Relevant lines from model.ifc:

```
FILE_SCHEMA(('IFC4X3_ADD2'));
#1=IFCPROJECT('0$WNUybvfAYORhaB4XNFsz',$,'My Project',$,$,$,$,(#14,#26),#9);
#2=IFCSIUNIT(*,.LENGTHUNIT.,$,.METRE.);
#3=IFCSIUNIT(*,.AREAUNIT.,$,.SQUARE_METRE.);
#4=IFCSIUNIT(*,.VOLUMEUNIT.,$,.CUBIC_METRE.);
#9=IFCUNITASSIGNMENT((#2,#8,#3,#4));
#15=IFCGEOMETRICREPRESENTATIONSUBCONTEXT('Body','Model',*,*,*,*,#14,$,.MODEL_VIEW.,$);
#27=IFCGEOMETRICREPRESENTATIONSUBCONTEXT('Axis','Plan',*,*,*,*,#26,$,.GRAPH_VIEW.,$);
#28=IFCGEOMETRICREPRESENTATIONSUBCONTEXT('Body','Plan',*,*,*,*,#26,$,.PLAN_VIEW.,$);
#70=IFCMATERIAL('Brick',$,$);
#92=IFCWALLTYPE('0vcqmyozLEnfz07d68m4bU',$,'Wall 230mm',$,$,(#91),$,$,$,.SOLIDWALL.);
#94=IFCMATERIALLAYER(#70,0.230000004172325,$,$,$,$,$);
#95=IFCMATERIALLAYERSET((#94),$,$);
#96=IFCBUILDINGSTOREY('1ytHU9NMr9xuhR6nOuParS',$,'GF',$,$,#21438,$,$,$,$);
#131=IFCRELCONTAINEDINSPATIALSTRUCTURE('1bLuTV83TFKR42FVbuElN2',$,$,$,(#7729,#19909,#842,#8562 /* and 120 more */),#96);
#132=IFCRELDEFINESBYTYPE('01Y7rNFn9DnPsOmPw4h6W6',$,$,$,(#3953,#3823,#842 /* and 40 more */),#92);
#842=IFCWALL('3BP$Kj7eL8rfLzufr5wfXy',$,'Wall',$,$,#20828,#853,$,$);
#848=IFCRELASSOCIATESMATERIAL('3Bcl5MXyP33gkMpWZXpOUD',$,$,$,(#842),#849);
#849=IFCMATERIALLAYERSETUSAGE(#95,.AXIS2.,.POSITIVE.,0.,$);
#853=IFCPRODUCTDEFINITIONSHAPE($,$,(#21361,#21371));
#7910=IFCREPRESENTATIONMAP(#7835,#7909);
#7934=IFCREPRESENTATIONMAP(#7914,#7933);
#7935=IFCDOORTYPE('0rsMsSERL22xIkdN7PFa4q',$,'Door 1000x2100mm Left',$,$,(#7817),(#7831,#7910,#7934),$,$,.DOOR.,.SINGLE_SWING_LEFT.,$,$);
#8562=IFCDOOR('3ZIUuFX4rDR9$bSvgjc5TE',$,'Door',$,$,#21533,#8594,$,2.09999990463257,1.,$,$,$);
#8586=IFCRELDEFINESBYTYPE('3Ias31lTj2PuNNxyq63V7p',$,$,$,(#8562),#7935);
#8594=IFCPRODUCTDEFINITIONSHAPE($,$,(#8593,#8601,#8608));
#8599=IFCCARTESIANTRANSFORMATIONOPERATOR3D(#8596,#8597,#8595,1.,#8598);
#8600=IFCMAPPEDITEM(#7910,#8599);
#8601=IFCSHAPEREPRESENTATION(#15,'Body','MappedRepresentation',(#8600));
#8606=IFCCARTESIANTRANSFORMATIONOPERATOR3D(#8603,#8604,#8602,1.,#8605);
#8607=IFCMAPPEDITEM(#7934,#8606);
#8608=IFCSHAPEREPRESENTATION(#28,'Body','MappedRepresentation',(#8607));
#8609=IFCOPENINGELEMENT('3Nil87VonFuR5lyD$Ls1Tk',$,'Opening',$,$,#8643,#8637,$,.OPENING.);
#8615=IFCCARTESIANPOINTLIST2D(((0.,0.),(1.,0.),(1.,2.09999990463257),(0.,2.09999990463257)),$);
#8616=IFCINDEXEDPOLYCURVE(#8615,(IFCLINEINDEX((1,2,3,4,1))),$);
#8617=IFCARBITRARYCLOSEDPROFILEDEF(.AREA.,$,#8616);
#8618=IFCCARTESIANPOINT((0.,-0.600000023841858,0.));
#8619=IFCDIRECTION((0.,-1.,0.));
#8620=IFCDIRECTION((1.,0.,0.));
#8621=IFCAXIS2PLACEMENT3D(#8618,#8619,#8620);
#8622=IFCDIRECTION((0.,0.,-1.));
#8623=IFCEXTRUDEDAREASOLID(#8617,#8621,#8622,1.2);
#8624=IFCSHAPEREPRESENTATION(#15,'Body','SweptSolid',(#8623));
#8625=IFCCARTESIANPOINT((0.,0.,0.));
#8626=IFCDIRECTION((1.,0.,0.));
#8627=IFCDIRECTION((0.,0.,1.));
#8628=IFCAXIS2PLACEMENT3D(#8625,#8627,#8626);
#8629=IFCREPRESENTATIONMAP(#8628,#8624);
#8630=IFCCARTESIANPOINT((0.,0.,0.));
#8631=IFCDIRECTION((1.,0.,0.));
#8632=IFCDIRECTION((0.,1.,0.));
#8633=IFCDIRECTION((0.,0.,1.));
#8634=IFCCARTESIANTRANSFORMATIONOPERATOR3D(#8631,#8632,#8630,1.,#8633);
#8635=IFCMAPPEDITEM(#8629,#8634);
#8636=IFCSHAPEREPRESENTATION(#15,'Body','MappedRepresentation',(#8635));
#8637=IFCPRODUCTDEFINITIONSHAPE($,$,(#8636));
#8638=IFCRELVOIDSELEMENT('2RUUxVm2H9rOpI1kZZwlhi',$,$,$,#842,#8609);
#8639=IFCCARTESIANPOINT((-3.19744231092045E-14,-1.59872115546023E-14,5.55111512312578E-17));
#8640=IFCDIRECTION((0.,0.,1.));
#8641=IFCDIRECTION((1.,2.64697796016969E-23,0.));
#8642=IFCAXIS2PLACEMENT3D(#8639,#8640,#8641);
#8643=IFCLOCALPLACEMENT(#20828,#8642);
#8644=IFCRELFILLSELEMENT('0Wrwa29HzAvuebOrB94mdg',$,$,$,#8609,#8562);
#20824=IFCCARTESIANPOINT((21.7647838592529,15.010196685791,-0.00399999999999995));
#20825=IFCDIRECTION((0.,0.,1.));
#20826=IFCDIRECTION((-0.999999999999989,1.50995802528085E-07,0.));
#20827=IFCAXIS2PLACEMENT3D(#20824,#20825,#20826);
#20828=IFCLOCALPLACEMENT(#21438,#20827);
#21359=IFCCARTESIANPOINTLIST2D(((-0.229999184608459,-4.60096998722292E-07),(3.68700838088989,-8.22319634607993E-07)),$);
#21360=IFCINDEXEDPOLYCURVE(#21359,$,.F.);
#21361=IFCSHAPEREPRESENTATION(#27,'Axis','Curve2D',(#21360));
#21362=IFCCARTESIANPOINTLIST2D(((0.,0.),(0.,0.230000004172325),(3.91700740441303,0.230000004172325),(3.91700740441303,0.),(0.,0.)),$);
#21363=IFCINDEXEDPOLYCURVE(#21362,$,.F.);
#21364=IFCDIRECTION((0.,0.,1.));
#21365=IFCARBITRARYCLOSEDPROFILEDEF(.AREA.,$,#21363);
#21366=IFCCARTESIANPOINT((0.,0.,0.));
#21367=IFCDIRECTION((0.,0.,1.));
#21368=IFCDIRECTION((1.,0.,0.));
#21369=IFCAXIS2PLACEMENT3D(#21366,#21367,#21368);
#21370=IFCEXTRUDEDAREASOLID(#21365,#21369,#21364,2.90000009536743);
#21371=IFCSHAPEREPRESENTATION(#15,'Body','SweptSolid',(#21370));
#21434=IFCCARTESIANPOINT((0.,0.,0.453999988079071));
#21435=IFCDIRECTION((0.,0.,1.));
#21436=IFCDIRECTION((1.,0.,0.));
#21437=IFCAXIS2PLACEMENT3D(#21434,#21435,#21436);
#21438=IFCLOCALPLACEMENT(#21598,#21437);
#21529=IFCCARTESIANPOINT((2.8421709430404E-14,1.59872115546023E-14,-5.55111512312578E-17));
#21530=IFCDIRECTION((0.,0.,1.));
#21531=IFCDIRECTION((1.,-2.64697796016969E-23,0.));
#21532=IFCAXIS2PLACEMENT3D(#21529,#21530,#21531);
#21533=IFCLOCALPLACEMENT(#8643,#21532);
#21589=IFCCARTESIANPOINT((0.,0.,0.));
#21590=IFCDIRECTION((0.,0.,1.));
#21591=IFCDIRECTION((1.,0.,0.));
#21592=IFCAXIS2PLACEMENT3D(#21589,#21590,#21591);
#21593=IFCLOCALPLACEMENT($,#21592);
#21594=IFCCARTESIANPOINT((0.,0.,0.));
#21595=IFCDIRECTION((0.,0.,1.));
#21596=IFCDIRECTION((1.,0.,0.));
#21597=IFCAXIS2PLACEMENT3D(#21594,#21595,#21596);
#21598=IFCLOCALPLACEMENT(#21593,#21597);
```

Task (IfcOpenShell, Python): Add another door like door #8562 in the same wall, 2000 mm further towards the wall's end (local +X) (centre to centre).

```python
import ifcopenshell
import ifcopenshell.api.feature
import ifcopenshell.api.geometry
import ifcopenshell.api.root
import ifcopenshell.geom
import ifcopenshell.util.element
import ifcopenshell.util.placement
import ifcopenshell.util.shape
import ifcopenshell.util.unit

model = ifcopenshell.open("model.ifc")
unit_scale = ifcopenshell.util.unit.calculate_unit_scale(model)
settings = ifcopenshell.geom.settings()


def volume(element):
    """Net volume in cubic metres, openings subtracted."""
    shape = ifcopenshell.geom.create_shape(settings, element)
    return ifcopenshell.util.shape.get_volume(shape.geometry)


door = model.by_guid("3ZIUuFX4rDR9$bSvgjc5TE")
opening = door.FillsVoids[0].RelatingOpeningElement
wall = opening.VoidsElements[0].RelatingBuildingElement
before = volume(wall)
shift = ifcopenshell.util.placement.get_local_placement(wall.ObjectPlacement)[:3, 0] * 2 / unit_scale

# copy_class copies the void relationship, type, container and properties, but no geometry.
new_opening = ifcopenshell.api.root.copy_class(model, product=opening)
new_opening.Representation = ifcopenshell.util.element.copy_deep(
    model, opening.Representation, exclude=["IfcGeometricRepresentationContext", "IfcRepresentationMap"]
)
new_door = ifcopenshell.api.root.copy_class(model, product=door)
new_door.Representation = ifcopenshell.util.element.copy_deep(
    model, door.Representation, exclude=["IfcGeometricRepresentationContext", "IfcRepresentationMap"]
)
ifcopenshell.api.feature.add_filling(model, opening=new_opening, element=new_door)

for old, new in ((opening, new_opening), (door, new_door)):
    matrix = ifcopenshell.util.placement.get_local_placement(old.ObjectPlacement)
    matrix[:3, 3] += shift
    ifcopenshell.api.geometry.edit_object_placement(model, product=new, matrix=matrix, is_si=False)

after = volume(wall)

print(f"wall volume {before:.3f} -> {after:.3f} m3")

model.write("model-out.ifc")
```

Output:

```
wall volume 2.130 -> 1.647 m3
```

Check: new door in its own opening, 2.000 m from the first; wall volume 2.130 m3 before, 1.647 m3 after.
